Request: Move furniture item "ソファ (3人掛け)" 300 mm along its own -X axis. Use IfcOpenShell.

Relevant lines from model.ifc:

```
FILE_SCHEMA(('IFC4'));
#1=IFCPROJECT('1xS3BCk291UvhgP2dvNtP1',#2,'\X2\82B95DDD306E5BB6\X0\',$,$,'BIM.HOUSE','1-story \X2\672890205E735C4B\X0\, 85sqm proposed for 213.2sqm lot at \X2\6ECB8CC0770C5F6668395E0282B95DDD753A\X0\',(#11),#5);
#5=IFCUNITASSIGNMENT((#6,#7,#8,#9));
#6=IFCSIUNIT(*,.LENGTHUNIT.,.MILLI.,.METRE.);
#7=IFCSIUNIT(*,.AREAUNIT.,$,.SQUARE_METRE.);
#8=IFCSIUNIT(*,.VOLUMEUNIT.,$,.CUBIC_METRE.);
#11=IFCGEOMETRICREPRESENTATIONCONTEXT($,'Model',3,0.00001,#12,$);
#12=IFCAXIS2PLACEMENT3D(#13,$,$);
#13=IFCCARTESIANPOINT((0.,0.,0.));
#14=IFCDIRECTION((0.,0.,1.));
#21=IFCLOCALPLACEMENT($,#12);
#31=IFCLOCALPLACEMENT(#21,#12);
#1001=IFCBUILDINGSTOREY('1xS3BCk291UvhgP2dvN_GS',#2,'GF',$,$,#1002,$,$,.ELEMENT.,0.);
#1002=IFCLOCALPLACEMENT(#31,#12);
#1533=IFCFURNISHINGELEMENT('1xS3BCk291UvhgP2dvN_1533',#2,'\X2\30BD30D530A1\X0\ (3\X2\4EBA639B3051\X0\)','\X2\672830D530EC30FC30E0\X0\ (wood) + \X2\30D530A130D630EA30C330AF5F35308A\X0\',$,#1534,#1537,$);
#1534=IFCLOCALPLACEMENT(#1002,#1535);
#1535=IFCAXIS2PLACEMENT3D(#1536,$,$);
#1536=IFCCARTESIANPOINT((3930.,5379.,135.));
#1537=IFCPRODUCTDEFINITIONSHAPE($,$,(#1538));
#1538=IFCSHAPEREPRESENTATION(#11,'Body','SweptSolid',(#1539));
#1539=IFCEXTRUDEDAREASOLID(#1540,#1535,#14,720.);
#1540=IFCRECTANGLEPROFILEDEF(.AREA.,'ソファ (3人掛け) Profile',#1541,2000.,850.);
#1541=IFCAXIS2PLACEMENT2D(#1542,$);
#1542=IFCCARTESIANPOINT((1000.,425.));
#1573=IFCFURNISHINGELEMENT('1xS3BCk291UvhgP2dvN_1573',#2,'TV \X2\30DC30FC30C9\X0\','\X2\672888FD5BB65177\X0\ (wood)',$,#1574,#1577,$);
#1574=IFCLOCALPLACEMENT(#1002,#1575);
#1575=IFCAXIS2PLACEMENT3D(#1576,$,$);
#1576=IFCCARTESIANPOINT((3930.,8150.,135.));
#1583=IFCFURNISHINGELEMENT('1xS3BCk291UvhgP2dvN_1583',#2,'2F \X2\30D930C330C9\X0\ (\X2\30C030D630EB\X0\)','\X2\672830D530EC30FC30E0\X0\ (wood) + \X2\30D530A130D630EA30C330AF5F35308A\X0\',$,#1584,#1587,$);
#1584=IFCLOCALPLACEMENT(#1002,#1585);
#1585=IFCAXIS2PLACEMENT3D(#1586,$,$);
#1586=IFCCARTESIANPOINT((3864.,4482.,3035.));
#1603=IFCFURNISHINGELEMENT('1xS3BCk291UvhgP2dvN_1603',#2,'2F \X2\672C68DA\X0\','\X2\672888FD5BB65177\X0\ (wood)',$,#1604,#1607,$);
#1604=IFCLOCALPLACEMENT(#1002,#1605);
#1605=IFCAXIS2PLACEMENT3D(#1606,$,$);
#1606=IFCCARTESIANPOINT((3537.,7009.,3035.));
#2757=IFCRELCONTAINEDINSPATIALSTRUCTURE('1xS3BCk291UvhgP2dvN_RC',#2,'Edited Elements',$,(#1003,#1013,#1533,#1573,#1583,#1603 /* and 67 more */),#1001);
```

```python
import ifcopenshell
import ifcopenshell.api.geometry
import ifcopenshell.util.placement
import ifcopenshell.util.unit

model = ifcopenshell.open("model.ifc")
unit_scale = ifcopenshell.util.unit.calculate_unit_scale(model)

item = model.by_guid("1xS3BCk291UvhgP2dvN_1533")
matrix = ifcopenshell.util.placement.get_local_placement(item.ObjectPlacement)
matrix[:3, 3] -= matrix[:3, 0] * 0.3 / unit_scale
ifcopenshell.api.geometry.edit_object_placement(model, product=item, matrix=matrix, is_si=False)

print(ifcopenshell.util.placement.get_local_placement(item.ObjectPlacement).round(3) + 0.0)

model.write("model_rev.ifc")
```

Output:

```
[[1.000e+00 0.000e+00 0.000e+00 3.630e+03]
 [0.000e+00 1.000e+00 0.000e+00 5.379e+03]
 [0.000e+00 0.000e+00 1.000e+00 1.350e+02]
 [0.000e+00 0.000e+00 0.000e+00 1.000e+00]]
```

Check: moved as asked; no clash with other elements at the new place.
